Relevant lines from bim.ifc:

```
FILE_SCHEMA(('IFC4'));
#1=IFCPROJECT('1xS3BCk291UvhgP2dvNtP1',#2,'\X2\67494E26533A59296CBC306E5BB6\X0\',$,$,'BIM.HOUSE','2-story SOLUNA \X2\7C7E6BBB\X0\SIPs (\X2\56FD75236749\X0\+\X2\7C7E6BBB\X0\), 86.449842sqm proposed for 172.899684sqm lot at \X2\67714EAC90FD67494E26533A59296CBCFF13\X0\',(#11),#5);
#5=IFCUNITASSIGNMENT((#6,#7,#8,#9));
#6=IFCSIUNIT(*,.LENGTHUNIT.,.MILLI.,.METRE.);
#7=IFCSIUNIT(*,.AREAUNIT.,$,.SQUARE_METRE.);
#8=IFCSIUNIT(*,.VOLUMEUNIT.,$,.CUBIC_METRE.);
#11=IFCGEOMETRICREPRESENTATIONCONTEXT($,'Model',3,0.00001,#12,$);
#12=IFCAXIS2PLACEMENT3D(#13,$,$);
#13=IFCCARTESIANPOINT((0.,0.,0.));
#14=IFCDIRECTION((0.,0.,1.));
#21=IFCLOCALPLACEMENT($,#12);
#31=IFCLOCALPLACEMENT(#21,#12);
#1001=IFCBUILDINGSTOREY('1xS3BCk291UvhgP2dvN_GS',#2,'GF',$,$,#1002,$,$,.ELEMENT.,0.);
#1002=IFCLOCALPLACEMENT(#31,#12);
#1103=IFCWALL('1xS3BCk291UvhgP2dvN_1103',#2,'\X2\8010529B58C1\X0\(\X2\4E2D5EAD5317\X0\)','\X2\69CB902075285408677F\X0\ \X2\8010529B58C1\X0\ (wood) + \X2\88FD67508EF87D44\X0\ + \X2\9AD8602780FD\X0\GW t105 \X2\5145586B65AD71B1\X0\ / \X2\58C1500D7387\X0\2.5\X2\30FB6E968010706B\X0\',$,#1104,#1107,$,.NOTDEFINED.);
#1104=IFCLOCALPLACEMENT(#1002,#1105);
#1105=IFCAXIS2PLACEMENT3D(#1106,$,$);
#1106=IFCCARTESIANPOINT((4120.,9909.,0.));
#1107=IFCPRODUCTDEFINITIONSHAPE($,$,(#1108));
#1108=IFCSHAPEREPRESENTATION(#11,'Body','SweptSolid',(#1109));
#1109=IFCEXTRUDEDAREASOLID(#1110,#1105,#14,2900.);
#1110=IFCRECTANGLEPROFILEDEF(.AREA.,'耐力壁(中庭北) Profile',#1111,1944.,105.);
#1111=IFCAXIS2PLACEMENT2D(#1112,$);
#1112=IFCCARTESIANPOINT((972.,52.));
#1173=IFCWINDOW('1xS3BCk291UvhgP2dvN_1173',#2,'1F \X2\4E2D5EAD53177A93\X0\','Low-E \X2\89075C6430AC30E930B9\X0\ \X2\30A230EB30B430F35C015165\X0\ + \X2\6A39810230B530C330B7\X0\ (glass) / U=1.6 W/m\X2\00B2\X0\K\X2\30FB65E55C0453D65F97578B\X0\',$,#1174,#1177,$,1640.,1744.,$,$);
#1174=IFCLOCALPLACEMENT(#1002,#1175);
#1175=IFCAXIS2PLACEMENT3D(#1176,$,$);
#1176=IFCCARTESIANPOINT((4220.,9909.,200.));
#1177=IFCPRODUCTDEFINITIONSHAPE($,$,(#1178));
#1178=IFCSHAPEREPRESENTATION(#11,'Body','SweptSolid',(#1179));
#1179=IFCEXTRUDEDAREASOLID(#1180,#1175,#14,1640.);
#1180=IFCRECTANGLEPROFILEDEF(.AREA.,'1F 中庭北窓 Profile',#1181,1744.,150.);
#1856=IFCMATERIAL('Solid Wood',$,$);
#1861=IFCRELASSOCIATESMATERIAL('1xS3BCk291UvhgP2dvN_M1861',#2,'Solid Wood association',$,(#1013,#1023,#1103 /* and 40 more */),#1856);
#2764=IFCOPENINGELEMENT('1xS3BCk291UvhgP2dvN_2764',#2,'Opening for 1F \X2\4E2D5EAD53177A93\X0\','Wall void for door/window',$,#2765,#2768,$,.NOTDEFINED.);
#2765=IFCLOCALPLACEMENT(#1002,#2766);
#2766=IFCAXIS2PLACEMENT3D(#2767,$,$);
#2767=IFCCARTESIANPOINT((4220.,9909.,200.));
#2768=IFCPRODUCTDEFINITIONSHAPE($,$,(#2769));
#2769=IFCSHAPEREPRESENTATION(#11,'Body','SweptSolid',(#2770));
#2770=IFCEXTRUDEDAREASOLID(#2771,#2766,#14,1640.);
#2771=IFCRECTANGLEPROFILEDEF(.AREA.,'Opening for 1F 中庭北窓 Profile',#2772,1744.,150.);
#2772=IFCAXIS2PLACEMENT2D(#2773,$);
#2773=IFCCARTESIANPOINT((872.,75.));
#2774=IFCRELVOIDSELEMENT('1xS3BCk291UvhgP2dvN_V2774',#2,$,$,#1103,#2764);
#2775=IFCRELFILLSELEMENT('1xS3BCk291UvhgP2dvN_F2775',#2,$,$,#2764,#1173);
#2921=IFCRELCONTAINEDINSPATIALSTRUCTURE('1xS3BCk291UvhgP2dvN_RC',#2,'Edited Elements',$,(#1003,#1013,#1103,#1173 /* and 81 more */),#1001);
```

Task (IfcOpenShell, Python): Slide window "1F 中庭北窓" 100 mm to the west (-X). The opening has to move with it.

```python
import ifcopenshell
import ifcopenshell.api.geometry
import ifcopenshell.util.placement
import ifcopenshell.util.unit

model = ifcopenshell.open("bim.ifc")
unit_scale = ifcopenshell.util.unit.calculate_unit_scale(model)

window = model.by_guid("1xS3BCk291UvhgP2dvN_1173")
opening = window.FillsVoids[0].RelatingOpeningElement
wall = opening.VoidsElements[0].RelatingBuildingElement

wall_matrix = ifcopenshell.util.placement.get_local_placement(wall.ObjectPlacement)
shift = wall_matrix[:3, 0] * -0.1 / unit_scale
before = ifcopenshell.util.placement.get_local_placement(window.ObjectPlacement)[:3, 3].copy()

# The window is not placed relative to its opening, so move both.
for product in (opening, window):
    matrix = ifcopenshell.util.placement.get_local_placement(product.ObjectPlacement)
    matrix[:3, 3] += shift
    ifcopenshell.api.geometry.edit_object_placement(model, product=product, matrix=matrix, is_si=False)

after = ifcopenshell.util.placement.get_local_placement(window.ObjectPlacement)[:3, 3]
print("window moved by", (after - before).round(3) + 0.0)

model.write("bim_rev.ifc")
```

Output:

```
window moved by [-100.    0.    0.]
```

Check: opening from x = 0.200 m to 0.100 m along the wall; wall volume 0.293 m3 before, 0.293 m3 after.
